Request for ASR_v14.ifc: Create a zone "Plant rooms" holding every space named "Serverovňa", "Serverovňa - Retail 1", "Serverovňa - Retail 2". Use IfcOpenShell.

First a look at what the model holds.

```python
import ifcopenshell

model = ifcopenshell.open("ASR_v14.ifc")
print(model.schema)
seen = {}
for space in model.by_type("IfcSpace"):
    seen[space.LongName] = seen.get(space.LongName, 0) + 1
for name, count in sorted(seen.items(), key=str):
    print(count, "x", name)
print("zones:", [z.Name for z in model.by_type("IfcZone")][:20])
```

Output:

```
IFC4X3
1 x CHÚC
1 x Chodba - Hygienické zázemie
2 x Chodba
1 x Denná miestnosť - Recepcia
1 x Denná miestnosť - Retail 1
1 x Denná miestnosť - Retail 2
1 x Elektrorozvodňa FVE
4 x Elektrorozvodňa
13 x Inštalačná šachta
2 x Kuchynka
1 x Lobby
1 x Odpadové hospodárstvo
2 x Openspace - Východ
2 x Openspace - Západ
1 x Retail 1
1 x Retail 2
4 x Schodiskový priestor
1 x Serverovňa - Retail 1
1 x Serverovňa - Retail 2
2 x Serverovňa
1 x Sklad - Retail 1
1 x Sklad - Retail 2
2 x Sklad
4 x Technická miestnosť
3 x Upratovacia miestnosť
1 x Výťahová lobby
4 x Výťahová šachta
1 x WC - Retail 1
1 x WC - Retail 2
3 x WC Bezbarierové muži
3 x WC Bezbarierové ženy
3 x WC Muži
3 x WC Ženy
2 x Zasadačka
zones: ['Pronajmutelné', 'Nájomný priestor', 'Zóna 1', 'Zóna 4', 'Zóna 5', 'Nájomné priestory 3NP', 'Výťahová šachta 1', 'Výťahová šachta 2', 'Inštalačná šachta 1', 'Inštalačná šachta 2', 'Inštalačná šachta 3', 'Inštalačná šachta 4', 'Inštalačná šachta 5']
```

```python
import ifcopenshell
import ifcopenshell.api.group
import ifcopenshell.api.root

model = ifcopenshell.open("ASR_v14.ifc")

names = {"Serverovňa", "Serverovňa - Retail 1", "Serverovňa - Retail 2"}
spaces = [s for s in model.by_type("IfcSpace") if s.LongName in names]

zone = ifcopenshell.api.root.create_entity(model, ifc_class="IfcZone", name="Plant rooms")
ifcopenshell.api.group.assign_group(model, products=spaces, group=zone)
print(len(spaces), "spaces in", zone.Name)

model.write("ASR_v14-out.ifc")
```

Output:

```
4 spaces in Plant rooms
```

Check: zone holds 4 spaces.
